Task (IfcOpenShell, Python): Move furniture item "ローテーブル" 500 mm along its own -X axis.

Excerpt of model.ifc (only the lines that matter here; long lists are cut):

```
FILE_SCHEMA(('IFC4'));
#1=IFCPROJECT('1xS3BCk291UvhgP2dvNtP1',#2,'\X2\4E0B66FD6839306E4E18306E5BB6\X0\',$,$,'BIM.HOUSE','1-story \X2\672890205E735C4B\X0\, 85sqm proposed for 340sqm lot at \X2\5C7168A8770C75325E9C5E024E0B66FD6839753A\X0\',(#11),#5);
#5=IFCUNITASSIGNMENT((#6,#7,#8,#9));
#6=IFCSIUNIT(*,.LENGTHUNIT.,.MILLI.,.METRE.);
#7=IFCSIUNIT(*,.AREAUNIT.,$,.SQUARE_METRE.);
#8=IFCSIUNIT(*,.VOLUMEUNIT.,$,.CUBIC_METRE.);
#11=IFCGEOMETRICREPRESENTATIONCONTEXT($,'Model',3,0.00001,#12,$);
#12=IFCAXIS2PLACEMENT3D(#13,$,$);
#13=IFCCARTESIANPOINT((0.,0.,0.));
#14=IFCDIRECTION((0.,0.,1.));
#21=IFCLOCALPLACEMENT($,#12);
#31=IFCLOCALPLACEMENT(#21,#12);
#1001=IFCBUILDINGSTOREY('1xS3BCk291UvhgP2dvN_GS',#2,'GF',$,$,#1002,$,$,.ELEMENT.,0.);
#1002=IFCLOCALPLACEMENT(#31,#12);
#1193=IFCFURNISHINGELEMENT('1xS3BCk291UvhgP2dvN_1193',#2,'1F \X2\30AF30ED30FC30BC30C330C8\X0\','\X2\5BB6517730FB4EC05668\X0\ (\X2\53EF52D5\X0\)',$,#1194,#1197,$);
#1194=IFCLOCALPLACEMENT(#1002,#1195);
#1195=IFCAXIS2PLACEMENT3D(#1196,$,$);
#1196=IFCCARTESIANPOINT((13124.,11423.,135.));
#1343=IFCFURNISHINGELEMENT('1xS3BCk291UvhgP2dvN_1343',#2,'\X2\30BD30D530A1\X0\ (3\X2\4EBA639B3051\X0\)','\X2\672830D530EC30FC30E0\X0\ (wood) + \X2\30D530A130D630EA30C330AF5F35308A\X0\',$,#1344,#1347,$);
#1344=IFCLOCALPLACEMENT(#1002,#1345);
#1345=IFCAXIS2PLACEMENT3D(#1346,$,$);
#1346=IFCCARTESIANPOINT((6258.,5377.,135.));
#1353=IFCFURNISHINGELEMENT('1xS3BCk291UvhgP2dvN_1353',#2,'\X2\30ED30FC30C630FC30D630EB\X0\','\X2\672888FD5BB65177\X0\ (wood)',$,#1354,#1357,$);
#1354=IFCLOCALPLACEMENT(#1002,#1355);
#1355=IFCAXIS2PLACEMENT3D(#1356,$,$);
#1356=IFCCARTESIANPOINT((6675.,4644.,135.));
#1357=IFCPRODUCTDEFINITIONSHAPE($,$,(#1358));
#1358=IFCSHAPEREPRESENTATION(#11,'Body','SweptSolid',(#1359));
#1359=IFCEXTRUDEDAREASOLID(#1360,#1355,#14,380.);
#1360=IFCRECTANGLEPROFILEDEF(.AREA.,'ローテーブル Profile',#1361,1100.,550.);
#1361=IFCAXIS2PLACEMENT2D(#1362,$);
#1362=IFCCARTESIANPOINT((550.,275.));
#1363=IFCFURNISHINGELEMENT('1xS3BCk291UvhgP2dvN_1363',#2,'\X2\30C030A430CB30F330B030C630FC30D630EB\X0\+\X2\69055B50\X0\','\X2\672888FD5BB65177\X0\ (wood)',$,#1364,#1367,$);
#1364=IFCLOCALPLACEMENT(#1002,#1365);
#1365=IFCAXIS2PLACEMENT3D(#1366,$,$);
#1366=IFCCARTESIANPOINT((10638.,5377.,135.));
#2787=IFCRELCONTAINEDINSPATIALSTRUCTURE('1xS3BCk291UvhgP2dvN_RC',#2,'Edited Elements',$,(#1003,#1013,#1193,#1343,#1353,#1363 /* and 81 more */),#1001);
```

```python
import ifcopenshell
import ifcopenshell.api.geometry
import ifcopenshell.util.placement
import ifcopenshell.util.unit

model = ifcopenshell.open("model.ifc")
unit_scale = ifcopenshell.util.unit.calculate_unit_scale(model)

item = model.by_guid("1xS3BCk291UvhgP2dvN_1353")
matrix = ifcopenshell.util.placement.get_local_placement(item.ObjectPlacement)
matrix[:3, 3] -= matrix[:3, 0] * 0.5 / unit_scale
ifcopenshell.api.geometry.edit_object_placement(model, product=item, matrix=matrix, is_si=False)

print(ifcopenshell.util.placement.get_local_placement(item.ObjectPlacement).round(3) + 0.0)

model.write("model_updated.ifc")
```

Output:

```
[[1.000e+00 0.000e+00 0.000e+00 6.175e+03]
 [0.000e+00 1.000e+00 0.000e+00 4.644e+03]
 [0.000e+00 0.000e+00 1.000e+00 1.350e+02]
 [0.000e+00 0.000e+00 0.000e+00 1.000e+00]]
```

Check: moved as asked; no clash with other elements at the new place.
